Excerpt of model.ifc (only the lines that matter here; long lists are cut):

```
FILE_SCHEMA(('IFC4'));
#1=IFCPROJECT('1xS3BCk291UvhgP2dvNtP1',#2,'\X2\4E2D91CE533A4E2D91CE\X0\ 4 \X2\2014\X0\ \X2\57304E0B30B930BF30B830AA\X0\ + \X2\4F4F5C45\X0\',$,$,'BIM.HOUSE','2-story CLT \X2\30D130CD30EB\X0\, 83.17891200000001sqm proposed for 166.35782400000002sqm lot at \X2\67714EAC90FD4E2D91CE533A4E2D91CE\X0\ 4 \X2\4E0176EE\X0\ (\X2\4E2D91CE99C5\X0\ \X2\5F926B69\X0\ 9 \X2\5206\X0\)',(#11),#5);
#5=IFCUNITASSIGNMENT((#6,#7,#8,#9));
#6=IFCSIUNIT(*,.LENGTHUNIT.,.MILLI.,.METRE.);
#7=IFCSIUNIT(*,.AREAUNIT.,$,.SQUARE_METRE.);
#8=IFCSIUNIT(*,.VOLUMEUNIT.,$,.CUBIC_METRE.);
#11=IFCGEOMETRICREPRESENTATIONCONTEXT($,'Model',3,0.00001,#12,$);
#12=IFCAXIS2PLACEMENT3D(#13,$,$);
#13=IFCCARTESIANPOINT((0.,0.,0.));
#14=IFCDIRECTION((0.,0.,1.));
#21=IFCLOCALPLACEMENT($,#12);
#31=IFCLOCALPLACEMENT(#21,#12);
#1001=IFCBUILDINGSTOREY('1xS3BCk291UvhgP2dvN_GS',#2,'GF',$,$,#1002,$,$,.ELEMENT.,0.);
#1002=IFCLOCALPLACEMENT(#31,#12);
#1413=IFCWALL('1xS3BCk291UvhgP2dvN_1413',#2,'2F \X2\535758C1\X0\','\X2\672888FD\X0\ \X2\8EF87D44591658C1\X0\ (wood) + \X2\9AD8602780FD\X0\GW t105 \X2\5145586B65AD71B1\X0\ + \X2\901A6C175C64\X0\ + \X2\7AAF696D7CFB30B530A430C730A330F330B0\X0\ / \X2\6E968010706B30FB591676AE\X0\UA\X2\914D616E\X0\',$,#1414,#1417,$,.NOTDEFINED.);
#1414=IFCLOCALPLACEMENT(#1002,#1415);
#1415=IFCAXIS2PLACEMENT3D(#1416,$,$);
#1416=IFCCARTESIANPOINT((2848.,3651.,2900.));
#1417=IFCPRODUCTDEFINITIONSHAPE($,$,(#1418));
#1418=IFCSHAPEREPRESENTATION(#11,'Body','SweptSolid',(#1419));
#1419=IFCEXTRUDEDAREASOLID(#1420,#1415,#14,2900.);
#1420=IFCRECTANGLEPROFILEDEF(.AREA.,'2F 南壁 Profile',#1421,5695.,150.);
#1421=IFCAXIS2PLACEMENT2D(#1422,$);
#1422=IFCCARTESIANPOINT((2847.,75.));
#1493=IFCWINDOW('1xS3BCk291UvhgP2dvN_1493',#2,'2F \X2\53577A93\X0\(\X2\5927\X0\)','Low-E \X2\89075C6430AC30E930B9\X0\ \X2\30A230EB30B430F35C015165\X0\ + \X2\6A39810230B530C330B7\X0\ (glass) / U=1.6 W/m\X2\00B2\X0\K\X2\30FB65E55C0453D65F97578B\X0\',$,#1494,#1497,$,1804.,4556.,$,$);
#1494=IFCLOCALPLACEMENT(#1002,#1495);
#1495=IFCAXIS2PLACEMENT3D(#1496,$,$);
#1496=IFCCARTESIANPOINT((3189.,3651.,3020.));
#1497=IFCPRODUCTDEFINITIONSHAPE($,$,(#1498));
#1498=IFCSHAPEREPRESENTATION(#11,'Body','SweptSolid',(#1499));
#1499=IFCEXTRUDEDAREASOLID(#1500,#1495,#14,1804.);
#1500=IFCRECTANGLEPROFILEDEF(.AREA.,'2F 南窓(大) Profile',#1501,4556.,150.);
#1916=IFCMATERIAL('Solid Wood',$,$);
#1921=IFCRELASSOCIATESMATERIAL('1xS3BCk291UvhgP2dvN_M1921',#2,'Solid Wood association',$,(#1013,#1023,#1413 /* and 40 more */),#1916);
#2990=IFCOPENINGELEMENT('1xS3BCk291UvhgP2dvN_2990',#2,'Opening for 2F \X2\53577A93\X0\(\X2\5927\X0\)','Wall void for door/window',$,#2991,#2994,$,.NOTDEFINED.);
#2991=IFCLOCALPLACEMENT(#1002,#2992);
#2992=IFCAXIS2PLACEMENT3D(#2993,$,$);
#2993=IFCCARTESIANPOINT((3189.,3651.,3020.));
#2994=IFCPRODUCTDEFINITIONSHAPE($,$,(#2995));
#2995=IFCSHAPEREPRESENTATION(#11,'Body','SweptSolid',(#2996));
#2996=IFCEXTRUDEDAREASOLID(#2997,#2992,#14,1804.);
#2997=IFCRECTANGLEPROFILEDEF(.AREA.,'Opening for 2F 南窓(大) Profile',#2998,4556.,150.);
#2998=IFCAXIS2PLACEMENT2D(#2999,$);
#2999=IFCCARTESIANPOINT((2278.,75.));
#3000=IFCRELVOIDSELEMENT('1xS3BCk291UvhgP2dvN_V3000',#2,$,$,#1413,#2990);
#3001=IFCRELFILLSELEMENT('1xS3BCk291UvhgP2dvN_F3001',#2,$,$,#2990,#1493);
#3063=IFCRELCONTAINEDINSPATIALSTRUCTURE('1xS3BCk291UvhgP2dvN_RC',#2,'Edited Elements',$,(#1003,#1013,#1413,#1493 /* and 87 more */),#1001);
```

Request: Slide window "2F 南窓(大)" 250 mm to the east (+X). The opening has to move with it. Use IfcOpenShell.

```python
import ifcopenshell
import ifcopenshell.api.geometry
import ifcopenshell.util.placement

model = ifcopenshell.open("model.ifc")

window = model.by_guid("1xS3BCk291UvhgP2dvN_1493")
opening = window.FillsVoids[0].RelatingOpeningElement
wall = opening.VoidsElements[0].RelatingBuildingElement

wall_matrix = ifcopenshell.util.placement.get_local_placement(wall.ObjectPlacement)
shift = wall_matrix[:3, 0] * 250.0
before = ifcopenshell.util.placement.get_local_placement(window.ObjectPlacement)[:3, 3].copy()

# The window is not placed relative to its opening, so move both.
for product in (opening, window):
    matrix = ifcopenshell.util.placement.get_local_placement(product.ObjectPlacement)
    matrix[:3, 3] += shift
    ifcopenshell.api.geometry.edit_object_placement(model, product=product, matrix=matrix, is_si=False)

after = ifcopenshell.util.placement.get_local_placement(window.ObjectPlacement)[:3, 3]
print("window moved by", (after - before).round(3) + 0.0)

model.write("model_v2.ifc")
```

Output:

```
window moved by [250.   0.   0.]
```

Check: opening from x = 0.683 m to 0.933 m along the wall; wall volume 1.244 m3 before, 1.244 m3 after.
